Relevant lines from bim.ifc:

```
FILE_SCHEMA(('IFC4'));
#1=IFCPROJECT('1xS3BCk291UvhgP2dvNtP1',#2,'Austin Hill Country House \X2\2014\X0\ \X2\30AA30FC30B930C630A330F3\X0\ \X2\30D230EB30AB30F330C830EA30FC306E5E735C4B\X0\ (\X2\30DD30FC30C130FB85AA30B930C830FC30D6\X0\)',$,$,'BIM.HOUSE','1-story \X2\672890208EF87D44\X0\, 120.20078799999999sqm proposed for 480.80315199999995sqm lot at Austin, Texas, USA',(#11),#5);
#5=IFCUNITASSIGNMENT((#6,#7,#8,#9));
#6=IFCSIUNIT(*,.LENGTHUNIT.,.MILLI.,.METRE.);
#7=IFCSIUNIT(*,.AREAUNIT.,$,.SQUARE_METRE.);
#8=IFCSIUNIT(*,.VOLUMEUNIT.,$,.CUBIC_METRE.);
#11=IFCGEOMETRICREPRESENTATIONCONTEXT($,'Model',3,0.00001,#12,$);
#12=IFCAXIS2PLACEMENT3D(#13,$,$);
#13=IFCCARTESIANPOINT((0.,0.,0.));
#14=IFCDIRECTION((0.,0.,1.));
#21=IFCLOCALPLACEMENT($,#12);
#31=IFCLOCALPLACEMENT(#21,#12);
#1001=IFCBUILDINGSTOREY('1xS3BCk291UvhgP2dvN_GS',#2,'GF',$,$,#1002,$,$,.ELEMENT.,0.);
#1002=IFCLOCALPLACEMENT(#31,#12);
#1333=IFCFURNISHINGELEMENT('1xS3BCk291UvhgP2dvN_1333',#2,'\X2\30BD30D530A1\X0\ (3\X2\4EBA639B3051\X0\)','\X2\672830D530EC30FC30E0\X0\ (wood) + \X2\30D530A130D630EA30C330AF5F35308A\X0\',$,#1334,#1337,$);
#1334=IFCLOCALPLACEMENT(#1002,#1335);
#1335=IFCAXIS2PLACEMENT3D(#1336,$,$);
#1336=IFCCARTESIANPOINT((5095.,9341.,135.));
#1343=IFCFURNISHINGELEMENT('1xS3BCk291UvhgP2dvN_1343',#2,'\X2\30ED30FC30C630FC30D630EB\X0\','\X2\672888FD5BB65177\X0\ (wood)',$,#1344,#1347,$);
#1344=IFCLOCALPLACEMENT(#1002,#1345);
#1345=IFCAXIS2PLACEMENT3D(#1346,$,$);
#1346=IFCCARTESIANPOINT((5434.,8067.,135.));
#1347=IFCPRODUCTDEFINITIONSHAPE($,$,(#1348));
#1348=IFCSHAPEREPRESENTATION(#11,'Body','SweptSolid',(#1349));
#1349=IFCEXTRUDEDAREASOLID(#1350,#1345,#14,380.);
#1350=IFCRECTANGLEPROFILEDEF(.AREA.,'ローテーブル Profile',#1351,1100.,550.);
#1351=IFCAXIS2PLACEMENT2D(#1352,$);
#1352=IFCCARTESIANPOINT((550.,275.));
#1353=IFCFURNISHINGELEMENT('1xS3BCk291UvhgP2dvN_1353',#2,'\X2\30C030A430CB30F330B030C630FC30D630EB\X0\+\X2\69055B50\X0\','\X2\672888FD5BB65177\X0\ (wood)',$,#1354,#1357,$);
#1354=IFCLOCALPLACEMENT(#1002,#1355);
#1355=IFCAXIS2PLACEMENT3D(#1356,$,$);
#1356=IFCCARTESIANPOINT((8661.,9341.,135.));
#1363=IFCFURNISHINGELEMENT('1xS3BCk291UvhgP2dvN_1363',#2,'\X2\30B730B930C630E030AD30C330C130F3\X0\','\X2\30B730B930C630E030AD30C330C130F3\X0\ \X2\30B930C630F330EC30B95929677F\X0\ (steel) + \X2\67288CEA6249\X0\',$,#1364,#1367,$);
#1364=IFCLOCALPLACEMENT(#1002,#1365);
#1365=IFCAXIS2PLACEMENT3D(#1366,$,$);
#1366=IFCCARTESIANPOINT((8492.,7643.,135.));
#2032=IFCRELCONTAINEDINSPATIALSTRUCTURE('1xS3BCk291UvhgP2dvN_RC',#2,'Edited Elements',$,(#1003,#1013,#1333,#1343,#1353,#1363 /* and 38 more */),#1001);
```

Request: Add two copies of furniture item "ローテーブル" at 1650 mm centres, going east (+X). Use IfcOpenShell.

```python
import numpy as np
import ifcopenshell
import ifcopenshell.api.geometry
import ifcopenshell.api.root
import ifcopenshell.util.element
import ifcopenshell.util.placement

model = ifcopenshell.open("bim.ifc")


def reuse_history(source, copy):
    """copy_class also copies each property set's owner history, people and application; keep the originals."""
    for rel in copy.IsDefinedBy:
        if rel.is_a("IfcRelDefinesByProperties") and (history := rel.RelatingPropertyDefinition.OwnerHistory):
            rel.RelatingPropertyDefinition.OwnerHistory = source.OwnerHistory
            ifcopenshell.util.element.remove_deep2(model, history)


source = model.by_guid("1xS3BCk291UvhgP2dvN_1343")
base = ifcopenshell.util.placement.get_local_placement(source.ObjectPlacement)
step = np.array([1.0, 0.0, 0.0]) * 1650.0

for i in range(1, 3):
    copy = ifcopenshell.api.root.copy_class(model, product=source)
    copy.Representation = ifcopenshell.util.element.copy_deep(
        model, source.Representation, exclude=["IfcGeometricRepresentationContext", "IfcRepresentationMap"]
    )
    reuse_history(source, copy)
    matrix = base.copy()
    matrix[:3, 3] += i * step
    print("added at", matrix[:3, 3].round(3) + 0.0)
    ifcopenshell.api.geometry.edit_object_placement(model, product=copy, matrix=matrix, is_si=False)

model.write("bim_rev.ifc")
```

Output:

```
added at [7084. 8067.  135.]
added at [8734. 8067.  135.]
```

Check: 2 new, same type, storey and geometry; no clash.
